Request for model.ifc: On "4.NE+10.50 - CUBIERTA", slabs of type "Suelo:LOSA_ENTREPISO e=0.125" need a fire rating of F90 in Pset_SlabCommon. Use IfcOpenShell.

First a look at what the model holds.

```python
import ifcopenshell
import ifcopenshell.util.element

model = ifcopenshell.open("model.ifc")
print(model.schema)
storey = next(s for s in model.by_type("IfcBuildingStorey") if s.Name == "4.NE+10.50 - CUBIERTA")
slabs = [e for e in ifcopenshell.util.element.get_decomposition(storey) if e.is_a("IfcSlab")]
seen = {}
for e in slabs:
    element_type = ifcopenshell.util.element.get_type(e)
    key = (element_type.Name if element_type != e and element_type else None, ifcopenshell.util.element.get_pset(e, "Pset_SlabCommon", "FireRating"))
    seen[key] = seen.get(key, 0) + 1
for (name, value), count in sorted(seen.items(), key=str):
    print(count, "x", name, "|", value)
```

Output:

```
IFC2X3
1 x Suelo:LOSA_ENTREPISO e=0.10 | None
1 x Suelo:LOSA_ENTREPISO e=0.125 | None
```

```python
import ifcopenshell
import ifcopenshell.api.pset
import ifcopenshell.util.element

model = ifcopenshell.open("model.ifc")

storey = next(s for s in model.by_type("IfcBuildingStorey") if s.Name == "4.NE+10.50 - CUBIERTA")
slabs = [e for e in ifcopenshell.util.element.get_decomposition(storey) if e.is_a("IfcSlab")]

count = 0
for e in slabs:
    element_type = ifcopenshell.util.element.get_type(e)
    if element_type in (None, e) or element_type.Name != "Suelo:LOSA_ENTREPISO e=0.125":
        continue
    # add_pset returns the element's existing set when there is one.
    pset = ifcopenshell.api.pset.add_pset(model, product=e, name="Pset_SlabCommon")
    ifcopenshell.api.pset.edit_pset(model, pset=pset, properties={"FireRating": "F90"})
    count += 1

print(count, "slabs updated")

model.write("model_edited.ifc")
```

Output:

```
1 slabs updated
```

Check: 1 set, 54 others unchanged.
